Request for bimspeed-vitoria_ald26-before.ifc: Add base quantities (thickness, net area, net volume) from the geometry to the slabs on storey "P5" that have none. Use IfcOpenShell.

First a look at what the model holds.

```python
import ifcopenshell
import ifcopenshell.util.element
import ifcopenshell.util.unit

model = ifcopenshell.open("bimspeed-vitoria_ald26-before.ifc")
print(model.schema)
for unit_type in ("LENGTHUNIT", "AREAUNIT", "VOLUMEUNIT"):
    print(unit_type, ifcopenshell.util.unit.calculate_unit_scale(model, unit_type))
storey = next(s for s in model.by_type("IfcBuildingStorey") if s.Name == "P5")
slabs = [e for e in ifcopenshell.util.element.get_decomposition(storey) if e.is_a("IfcSlab")]
for e in sorted(slabs, key=lambda e: e.id()):
    print(e.id(), e.is_a(), e.Name, list(ifcopenshell.util.element.get_psets(e, qtos_only=True)), sep=" | ")
```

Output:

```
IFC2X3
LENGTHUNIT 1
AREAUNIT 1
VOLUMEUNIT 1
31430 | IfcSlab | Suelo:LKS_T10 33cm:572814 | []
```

```python
import ifcopenshell
import ifcopenshell.api.pset
import ifcopenshell.geom
import ifcopenshell.util.element
import ifcopenshell.util.shape
import ifcopenshell.util.unit

model = ifcopenshell.open("bimspeed-vitoria_ald26-before.ifc")
unit_scale = ifcopenshell.util.unit.calculate_unit_scale(model)
area_scale = ifcopenshell.util.unit.calculate_unit_scale(model, "AREAUNIT")
volume_scale = ifcopenshell.util.unit.calculate_unit_scale(model, "VOLUMEUNIT")
settings = ifcopenshell.geom.settings()

storey = next(s for s in model.by_type("IfcBuildingStorey") if s.Name == "P5")
slabs = [e for e in ifcopenshell.util.element.get_decomposition(storey) if e.is_a("IfcSlab")]

for e in sorted(slabs, key=lambda e: e.id()):
    if ifcopenshell.util.element.get_psets(e, qtos_only=True, should_inherit=False):
        continue
    # Geometry comes back in metres, in the element's own axes.
    shape = ifcopenshell.geom.create_shape(settings, e)
    values = {
        "Width": ifcopenshell.util.shape.get_z(shape.geometry) / unit_scale,
        "NetArea": ifcopenshell.util.shape.get_footprint_area(shape.geometry) / area_scale,
        "NetVolume": ifcopenshell.util.shape.get_volume(shape.geometry) / volume_scale,
    }
    qto = ifcopenshell.api.pset.add_qto(model, product=e, name="BaseQuantities")
    ifcopenshell.api.pset.edit_qto(model, qto=qto, properties=values)
    print(e.id(), {k: round(v, 3) for k, v in values.items()})

model.write("bimspeed-vitoria_ald26-before_v2.ifc")
```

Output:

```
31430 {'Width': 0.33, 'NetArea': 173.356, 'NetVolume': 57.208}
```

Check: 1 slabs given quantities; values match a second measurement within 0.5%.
